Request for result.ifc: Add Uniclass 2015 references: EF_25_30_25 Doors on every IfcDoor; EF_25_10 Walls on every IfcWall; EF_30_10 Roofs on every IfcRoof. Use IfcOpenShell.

First a look at what the model holds.

```python
import ifcopenshell

model = ifcopenshell.open("result.ifc")
print(model.schema)
print("classifications:", [c.Name for c in model.by_type("IfcClassification")])
for ifc_class in ("IfcDoor", "IfcRoof", "IfcStair", "IfcWall", "IfcWindow"):
    print(ifc_class, len(model.by_type(ifc_class)))
```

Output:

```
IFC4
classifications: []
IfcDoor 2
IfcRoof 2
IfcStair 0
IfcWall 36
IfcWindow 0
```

```python
import ifcopenshell
import ifcopenshell.api.classification

model = ifcopenshell.open("result.ifc")

system = ifcopenshell.api.classification.add_classification(model, classification="Uniclass 2015")

codes = {
    "IfcDoor": ("EF_25_30_25", "Doors"),
    "IfcWall": ("EF_25_10", "Walls"),
    "IfcRoof": ("EF_30_10", "Roofs"),
}
for ifc_class, (code, name) in codes.items():
    products = model.by_type(ifc_class)
    ifcopenshell.api.classification.add_reference(
        model, products=products, classification=system, identification=code, name=name
    )
    print(code, len(products))

model.write("result_updated.ifc")
```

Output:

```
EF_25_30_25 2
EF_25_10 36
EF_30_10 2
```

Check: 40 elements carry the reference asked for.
